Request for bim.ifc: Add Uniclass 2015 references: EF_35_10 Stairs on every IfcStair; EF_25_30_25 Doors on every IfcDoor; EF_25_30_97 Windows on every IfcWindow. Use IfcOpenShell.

First a look at what the model holds.

```python
import ifcopenshell

model = ifcopenshell.open("bim.ifc")
print(model.schema)
print("classifications:", [c.Name for c in model.by_type("IfcClassification")])
for ifc_class in ("IfcDoor", "IfcRoof", "IfcStair", "IfcWall", "IfcWindow"):
    print(ifc_class, len(model.by_type(ifc_class)))
```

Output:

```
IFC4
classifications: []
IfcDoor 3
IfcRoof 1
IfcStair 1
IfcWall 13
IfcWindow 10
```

```python
import ifcopenshell
import ifcopenshell.api.classification

model = ifcopenshell.open("bim.ifc")

system = ifcopenshell.api.classification.add_classification(model, classification="Uniclass 2015")

codes = {
    "IfcStair": ("EF_35_10", "Stairs"),
    "IfcDoor": ("EF_25_30_25", "Doors"),
    "IfcWindow": ("EF_25_30_97", "Windows"),
}
for ifc_class, (code, name) in codes.items():
    products = model.by_type(ifc_class)
    ifcopenshell.api.classification.add_reference(
        model, products=products, classification=system, identification=code, name=name
    )
    print(code, len(products))

model.write("bim_v2.ifc")
```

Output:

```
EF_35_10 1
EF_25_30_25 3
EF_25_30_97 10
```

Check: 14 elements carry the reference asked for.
